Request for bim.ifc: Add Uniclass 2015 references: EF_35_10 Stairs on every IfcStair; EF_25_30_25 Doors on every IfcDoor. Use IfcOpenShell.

First a look at what the model holds.

```python
import ifcopenshell

model = ifcopenshell.open("bim.ifc")
print(model.schema)
print("classifications:", [c.Name for c in model.by_type("IfcClassification")])
for ifc_class in ("IfcDoor", "IfcRoof", "IfcStair", "IfcWall", "IfcWindow"):
    print(ifc_class, len(model.by_type(ifc_class)))
```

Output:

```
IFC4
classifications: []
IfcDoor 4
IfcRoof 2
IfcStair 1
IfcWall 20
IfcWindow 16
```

```python
import ifcopenshell
import ifcopenshell.api.classification

model = ifcopenshell.open("bim.ifc")

system = ifcopenshell.api.classification.add_classification(model, classification="Uniclass 2015")

codes = {
    "IfcStair": ("EF_35_10", "Stairs"),
    "IfcDoor": ("EF_25_30_25", "Doors"),
}
for ifc_class, (code, name) in codes.items():
    products = model.by_type(ifc_class)
    ifcopenshell.api.classification.add_reference(
        model, products=products, classification=system, identification=code, name=name
    )
    print(code, len(products))

model.write("bim-out.ifc")
```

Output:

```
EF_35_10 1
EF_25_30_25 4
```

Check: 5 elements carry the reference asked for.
